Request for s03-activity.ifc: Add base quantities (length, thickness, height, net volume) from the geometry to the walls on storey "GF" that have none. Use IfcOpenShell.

First a look at what the model holds.

```python
import ifcopenshell
import ifcopenshell.util.element
import ifcopenshell.util.unit

model = ifcopenshell.open("s03-activity.ifc")
print(model.schema)
for unit_type in ("LENGTHUNIT", "AREAUNIT", "VOLUMEUNIT"):
    print(unit_type, ifcopenshell.util.unit.calculate_unit_scale(model, unit_type))
storey = next(s for s in model.by_type("IfcBuildingStorey") if s.Name == "GF")
walls = [e for e in ifcopenshell.util.element.get_decomposition(storey) if e.is_a("IfcWall")]
for e in sorted(walls, key=lambda e: e.id()):
    print(e.id(), e.is_a(), e.Name, list(ifcopenshell.util.element.get_psets(e, qtos_only=True)), sep=" | ")
```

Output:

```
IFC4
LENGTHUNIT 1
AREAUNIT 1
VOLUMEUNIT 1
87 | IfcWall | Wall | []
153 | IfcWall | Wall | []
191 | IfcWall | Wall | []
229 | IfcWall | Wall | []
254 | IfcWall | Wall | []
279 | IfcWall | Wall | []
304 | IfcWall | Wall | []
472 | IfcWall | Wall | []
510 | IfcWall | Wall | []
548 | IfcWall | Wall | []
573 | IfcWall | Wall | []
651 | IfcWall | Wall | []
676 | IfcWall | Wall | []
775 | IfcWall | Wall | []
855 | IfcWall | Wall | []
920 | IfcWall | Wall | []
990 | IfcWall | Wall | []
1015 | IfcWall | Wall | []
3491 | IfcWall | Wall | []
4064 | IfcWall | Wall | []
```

```python
import ifcopenshell
import ifcopenshell.api.pset
import ifcopenshell.geom
import ifcopenshell.util.element
import ifcopenshell.util.shape
import ifcopenshell.util.unit

model = ifcopenshell.open("s03-activity.ifc")
unit_scale = ifcopenshell.util.unit.calculate_unit_scale(model)
volume_scale = ifcopenshell.util.unit.calculate_unit_scale(model, "VOLUMEUNIT")
settings = ifcopenshell.geom.settings()

storey = next(s for s in model.by_type("IfcBuildingStorey") if s.Name == "GF")
walls = [e for e in ifcopenshell.util.element.get_decomposition(storey) if e.is_a("IfcWall")]

for e in sorted(walls, key=lambda e: e.id()):
    if ifcopenshell.util.element.get_psets(e, qtos_only=True, should_inherit=False):
        continue
    # Geometry comes back in metres, in the element's own axes.
    shape = ifcopenshell.geom.create_shape(settings, e)
    values = {
        "Length": ifcopenshell.util.shape.get_x(shape.geometry) / unit_scale,
        "Width": ifcopenshell.util.shape.get_y(shape.geometry) / unit_scale,
        "Height": ifcopenshell.util.shape.get_z(shape.geometry) / unit_scale,
        "NetVolume": ifcopenshell.util.shape.get_volume(shape.geometry) / volume_scale,
    }
    qto = ifcopenshell.api.pset.add_qto(model, product=e, name="Qto_WallBaseQuantities")
    ifcopenshell.api.pset.edit_qto(model, qto=qto, properties=values)
    print(e.id(), {k: round(v, 3) for k, v in values.items()})

model.write("s03-activity_updated.ifc")
```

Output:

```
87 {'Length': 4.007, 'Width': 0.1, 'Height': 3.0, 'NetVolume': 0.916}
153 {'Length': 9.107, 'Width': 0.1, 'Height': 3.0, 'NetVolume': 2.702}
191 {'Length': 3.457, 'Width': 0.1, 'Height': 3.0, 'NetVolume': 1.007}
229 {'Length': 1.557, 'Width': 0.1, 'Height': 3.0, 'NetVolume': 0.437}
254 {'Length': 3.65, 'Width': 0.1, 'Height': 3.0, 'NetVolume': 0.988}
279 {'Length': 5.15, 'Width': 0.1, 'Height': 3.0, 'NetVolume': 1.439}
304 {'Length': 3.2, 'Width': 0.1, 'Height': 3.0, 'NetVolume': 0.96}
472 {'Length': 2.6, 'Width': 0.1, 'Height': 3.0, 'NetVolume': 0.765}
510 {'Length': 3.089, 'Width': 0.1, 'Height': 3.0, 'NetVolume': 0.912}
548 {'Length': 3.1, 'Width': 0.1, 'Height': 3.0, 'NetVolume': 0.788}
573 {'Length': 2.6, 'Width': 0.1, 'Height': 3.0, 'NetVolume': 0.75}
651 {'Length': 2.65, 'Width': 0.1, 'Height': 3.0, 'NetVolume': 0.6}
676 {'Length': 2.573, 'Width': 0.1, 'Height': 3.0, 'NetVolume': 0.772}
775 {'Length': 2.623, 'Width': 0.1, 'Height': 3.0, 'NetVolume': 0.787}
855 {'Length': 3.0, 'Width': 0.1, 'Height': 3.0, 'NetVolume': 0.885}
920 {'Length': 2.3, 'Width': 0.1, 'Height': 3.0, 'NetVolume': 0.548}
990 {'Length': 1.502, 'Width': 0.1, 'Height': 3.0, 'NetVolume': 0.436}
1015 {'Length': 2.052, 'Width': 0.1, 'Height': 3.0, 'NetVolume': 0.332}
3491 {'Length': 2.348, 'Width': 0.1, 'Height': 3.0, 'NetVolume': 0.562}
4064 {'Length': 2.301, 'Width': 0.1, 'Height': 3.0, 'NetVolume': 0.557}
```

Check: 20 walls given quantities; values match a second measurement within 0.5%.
